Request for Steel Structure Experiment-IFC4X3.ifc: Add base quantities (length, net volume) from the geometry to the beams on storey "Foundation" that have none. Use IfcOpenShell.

First a look at what the model holds.

```python
import ifcopenshell
import ifcopenshell.util.element
import ifcopenshell.util.unit

model = ifcopenshell.open("Steel Structure Experiment-IFC4X3.ifc")
print(model.schema)
for unit_type in ("LENGTHUNIT", "AREAUNIT", "VOLUMEUNIT"):
    print(unit_type, ifcopenshell.util.unit.calculate_unit_scale(model, unit_type))
storey = next(s for s in model.by_type("IfcBuildingStorey") if s.Name == "Foundation")
beams = [e for e in ifcopenshell.util.element.get_decomposition(storey) if e.is_a("IfcBeam")]
for e in sorted(beams, key=lambda e: e.id()):
    print(e.id(), e.is_a(), e.Name, list(ifcopenshell.util.element.get_psets(e, qtos_only=True)), sep=" | ")
```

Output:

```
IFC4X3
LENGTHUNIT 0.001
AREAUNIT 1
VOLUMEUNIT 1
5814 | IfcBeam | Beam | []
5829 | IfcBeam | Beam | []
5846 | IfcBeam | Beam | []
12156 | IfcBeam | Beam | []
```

```python
import ifcopenshell
import ifcopenshell.api.pset
import ifcopenshell.geom
import ifcopenshell.util.element
import ifcopenshell.util.shape
import ifcopenshell.util.unit

model = ifcopenshell.open("Steel Structure Experiment-IFC4X3.ifc")
unit_scale = ifcopenshell.util.unit.calculate_unit_scale(model)
volume_scale = ifcopenshell.util.unit.calculate_unit_scale(model, "VOLUMEUNIT")
settings = ifcopenshell.geom.settings()

storey = next(s for s in model.by_type("IfcBuildingStorey") if s.Name == "Foundation")
beams = [e for e in ifcopenshell.util.element.get_decomposition(storey) if e.is_a("IfcBeam")]

for e in sorted(beams, key=lambda e: e.id()):
    if ifcopenshell.util.element.get_psets(e, qtos_only=True, should_inherit=False):
        continue
    # Geometry comes back in metres, in the element's own axes.
    shape = ifcopenshell.geom.create_shape(settings, e)
    values = {
        "Length": ifcopenshell.util.shape.get_max_xyz(shape.geometry) / unit_scale,
        "NetVolume": ifcopenshell.util.shape.get_volume(shape.geometry) / volume_scale,
    }
    qto = ifcopenshell.api.pset.add_qto(model, product=e, name="Qto_BeamBaseQuantities")
    ifcopenshell.api.pset.edit_qto(model, qto=qto, properties=values)
    print(e.id(), {k: round(v, 3) for k, v in values.items()})

model.write("Steel Structure Experiment-IFC4X3-out.ifc")
```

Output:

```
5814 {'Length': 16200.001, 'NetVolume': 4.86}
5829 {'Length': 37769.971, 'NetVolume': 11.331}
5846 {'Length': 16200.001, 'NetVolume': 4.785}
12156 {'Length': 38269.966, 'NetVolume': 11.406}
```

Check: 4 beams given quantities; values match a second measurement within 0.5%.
